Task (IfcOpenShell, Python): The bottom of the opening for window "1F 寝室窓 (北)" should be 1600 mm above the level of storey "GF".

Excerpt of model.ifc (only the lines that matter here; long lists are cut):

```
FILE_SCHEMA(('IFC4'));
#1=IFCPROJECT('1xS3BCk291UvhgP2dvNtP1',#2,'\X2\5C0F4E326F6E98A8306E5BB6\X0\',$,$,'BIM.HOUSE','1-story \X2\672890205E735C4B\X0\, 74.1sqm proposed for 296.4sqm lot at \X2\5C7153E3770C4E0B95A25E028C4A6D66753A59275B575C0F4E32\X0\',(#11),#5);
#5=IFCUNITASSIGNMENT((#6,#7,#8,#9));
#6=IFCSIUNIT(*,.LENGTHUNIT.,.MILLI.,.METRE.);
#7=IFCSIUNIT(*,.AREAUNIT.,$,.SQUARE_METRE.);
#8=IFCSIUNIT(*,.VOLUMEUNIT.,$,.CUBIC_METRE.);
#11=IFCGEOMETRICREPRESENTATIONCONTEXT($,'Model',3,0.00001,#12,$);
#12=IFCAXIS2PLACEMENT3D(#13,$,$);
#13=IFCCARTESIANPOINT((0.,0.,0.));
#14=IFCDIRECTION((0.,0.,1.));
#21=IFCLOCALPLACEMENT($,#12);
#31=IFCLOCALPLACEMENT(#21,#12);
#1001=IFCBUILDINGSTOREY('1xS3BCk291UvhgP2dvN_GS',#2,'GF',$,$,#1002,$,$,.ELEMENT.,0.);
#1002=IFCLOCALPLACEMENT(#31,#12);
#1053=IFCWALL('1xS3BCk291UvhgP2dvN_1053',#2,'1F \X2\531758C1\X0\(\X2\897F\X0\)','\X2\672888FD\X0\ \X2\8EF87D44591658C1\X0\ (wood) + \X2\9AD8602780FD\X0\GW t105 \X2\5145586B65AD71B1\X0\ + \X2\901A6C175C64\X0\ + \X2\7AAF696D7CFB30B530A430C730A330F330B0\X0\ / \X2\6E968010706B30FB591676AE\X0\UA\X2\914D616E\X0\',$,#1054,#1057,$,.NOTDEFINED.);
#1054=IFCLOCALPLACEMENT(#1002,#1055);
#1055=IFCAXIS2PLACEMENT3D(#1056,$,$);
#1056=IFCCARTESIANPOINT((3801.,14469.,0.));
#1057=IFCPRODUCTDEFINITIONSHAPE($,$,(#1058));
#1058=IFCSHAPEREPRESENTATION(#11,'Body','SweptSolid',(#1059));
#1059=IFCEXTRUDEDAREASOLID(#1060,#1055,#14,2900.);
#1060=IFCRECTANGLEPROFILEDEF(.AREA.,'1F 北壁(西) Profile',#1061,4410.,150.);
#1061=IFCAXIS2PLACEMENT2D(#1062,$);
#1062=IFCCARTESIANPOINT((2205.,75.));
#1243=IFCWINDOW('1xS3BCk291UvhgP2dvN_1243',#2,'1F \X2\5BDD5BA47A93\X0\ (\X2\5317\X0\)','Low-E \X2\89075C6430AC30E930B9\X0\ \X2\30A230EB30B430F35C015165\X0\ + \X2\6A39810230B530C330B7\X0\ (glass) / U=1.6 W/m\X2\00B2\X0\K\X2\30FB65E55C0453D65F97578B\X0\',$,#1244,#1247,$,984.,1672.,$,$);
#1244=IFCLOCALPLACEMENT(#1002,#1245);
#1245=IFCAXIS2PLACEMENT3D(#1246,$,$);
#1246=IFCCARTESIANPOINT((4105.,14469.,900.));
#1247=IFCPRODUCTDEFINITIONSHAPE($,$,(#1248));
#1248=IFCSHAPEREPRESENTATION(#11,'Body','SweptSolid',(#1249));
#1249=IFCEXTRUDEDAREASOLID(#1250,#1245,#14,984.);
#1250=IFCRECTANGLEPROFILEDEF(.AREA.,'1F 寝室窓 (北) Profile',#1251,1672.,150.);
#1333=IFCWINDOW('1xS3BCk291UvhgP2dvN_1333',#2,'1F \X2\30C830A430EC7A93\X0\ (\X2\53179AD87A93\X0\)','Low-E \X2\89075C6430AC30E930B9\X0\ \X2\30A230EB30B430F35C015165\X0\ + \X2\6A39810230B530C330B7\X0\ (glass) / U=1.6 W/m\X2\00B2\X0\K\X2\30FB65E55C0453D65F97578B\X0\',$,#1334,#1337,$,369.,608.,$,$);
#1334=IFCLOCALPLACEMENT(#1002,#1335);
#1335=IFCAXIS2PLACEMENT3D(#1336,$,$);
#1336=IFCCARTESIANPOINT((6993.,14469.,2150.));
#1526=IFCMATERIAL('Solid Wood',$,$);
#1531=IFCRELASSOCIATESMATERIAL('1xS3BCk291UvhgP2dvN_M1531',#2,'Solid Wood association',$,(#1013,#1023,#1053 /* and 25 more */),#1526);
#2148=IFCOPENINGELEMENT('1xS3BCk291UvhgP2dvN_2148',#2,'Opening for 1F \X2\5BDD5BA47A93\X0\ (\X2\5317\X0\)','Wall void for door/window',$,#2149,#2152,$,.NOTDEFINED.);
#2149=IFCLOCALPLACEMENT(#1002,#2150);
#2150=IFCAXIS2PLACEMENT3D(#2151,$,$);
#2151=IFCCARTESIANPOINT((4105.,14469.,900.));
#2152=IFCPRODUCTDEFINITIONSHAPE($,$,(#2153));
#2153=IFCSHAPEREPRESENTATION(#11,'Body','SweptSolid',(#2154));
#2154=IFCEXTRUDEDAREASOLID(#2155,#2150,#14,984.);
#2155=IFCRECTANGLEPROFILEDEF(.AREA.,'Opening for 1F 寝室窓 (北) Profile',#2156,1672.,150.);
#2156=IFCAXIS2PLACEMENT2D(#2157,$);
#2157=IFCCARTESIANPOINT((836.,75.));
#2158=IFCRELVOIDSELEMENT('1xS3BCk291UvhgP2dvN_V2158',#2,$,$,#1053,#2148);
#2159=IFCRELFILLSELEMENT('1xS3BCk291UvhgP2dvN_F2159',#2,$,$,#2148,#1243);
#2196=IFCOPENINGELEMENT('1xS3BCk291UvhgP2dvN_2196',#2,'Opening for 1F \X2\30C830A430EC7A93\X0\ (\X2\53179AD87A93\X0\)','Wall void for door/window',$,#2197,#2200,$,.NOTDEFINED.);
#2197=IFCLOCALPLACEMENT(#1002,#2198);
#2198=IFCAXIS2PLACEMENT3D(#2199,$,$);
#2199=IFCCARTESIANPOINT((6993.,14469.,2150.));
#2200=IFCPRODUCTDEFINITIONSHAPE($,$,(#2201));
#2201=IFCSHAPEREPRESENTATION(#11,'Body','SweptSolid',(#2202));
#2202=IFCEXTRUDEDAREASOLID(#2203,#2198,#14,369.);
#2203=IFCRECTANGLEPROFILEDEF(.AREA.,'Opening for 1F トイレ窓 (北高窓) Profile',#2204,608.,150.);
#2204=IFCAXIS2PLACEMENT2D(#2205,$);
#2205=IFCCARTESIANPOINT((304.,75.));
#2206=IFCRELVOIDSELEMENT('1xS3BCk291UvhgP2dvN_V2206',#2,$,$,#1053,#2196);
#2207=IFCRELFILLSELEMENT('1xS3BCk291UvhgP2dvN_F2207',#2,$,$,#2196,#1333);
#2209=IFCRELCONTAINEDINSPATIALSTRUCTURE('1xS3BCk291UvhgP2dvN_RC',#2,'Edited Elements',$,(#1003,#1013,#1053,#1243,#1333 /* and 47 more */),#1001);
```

```python
import numpy as np
import ifcopenshell
import ifcopenshell.api.geometry
import ifcopenshell.geom
import ifcopenshell.util.element
import ifcopenshell.util.placement
import ifcopenshell.util.shape
import ifcopenshell.util.unit

model = ifcopenshell.open("model.ifc")
unit_scale = ifcopenshell.util.unit.calculate_unit_scale(model)

window = model.by_id(1243)
opening = window.FillsVoids[0].RelatingOpeningElement
storey = ifcopenshell.util.element.get_container(window, ifc_class="IfcBuildingStorey")
level = ifcopenshell.util.placement.get_local_placement(storey.ObjectPlacement)[2, 3]

# The opening's origin need not be at the sill, so measure its lowest point.
shape = ifcopenshell.geom.create_shape(ifcopenshell.geom.settings(), opening)
bottom = ifcopenshell.util.shape.get_shape_bottom_elevation(shape, shape.geometry) / unit_scale
dz = level + 1600.0 - bottom

shift = np.array([0.0, 0.0, dz])
# The window is not placed relative to its opening, so move both.
for product in (opening, window):
    matrix = ifcopenshell.util.placement.get_local_placement(product.ObjectPlacement)
    matrix[:3, 3] += shift
    ifcopenshell.api.geometry.edit_object_placement(model, product=product, matrix=matrix, is_si=False)

print(f"moved by {dz * unit_scale:+.3f} m")

model.write("model_v2.ifc")
```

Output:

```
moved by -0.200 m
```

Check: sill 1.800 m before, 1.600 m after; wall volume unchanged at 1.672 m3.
